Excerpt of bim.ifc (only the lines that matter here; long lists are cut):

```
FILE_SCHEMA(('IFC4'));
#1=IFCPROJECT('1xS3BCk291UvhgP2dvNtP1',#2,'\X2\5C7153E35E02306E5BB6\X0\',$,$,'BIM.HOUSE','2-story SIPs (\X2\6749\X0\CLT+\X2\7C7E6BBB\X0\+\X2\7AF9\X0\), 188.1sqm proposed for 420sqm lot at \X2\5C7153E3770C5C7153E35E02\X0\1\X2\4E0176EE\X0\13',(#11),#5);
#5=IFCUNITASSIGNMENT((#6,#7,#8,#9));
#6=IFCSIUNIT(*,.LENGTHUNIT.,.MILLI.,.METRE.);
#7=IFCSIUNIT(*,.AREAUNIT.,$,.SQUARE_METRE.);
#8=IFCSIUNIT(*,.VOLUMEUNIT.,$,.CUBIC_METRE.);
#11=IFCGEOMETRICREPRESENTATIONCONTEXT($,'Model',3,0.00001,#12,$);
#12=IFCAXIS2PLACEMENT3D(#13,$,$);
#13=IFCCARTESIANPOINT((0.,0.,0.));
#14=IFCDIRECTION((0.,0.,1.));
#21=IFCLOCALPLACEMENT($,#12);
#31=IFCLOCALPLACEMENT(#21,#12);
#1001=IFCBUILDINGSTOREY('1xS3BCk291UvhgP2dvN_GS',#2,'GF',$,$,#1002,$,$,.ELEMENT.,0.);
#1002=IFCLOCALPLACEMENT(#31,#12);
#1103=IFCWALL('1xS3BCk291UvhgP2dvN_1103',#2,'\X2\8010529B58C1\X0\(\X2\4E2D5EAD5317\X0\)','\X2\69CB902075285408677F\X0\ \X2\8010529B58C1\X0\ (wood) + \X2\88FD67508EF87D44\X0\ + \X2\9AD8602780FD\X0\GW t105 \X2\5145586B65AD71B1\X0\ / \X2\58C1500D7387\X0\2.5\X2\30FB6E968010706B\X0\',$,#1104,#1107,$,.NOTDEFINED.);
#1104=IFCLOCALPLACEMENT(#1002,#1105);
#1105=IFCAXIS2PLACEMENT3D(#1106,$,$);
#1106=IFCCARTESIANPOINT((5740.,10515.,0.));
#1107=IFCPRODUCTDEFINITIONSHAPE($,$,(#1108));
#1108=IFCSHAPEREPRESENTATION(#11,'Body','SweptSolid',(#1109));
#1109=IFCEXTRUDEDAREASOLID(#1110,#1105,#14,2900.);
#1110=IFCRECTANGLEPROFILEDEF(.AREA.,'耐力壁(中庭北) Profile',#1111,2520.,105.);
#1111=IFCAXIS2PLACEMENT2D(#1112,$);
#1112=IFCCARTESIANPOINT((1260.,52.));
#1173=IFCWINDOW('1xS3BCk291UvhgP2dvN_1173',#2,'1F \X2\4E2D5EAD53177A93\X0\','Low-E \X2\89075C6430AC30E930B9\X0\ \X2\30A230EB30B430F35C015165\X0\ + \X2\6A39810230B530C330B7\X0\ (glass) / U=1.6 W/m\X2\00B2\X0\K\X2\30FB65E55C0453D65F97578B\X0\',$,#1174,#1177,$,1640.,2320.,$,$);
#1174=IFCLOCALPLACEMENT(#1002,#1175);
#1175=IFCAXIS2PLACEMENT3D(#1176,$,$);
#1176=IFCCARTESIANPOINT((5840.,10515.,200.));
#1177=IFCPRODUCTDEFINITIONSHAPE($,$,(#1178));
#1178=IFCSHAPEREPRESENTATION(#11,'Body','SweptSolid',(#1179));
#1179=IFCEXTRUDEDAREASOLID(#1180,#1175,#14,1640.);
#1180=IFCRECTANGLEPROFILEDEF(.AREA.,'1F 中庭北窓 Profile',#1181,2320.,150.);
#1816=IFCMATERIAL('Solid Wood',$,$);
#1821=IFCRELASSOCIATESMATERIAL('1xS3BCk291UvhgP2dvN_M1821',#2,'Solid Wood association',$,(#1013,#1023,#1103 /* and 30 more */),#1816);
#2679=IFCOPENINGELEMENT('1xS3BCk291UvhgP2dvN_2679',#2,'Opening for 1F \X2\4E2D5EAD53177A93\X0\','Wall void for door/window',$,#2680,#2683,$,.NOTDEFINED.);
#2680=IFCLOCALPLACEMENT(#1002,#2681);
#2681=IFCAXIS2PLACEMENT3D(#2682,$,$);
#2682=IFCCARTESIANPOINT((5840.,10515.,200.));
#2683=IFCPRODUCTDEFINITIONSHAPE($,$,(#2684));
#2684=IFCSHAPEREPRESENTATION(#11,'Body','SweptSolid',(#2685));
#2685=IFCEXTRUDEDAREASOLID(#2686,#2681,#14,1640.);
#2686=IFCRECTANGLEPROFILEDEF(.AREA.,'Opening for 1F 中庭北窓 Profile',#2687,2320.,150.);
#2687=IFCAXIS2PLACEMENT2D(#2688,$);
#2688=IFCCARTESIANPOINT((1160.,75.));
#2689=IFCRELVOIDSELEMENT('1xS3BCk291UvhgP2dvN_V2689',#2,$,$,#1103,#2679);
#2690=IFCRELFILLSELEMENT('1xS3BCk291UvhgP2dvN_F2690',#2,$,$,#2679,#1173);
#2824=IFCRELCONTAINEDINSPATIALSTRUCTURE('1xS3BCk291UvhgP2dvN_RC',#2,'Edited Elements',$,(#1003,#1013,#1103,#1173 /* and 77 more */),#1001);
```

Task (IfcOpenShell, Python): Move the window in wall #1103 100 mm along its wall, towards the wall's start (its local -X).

```python
import ifcopenshell
import ifcopenshell.api.geometry
import ifcopenshell.util.placement
import ifcopenshell.util.unit

model = ifcopenshell.open("bim.ifc")
unit_scale = ifcopenshell.util.unit.calculate_unit_scale(model)

window = model.by_guid("1xS3BCk291UvhgP2dvN_1173")
opening = window.FillsVoids[0].RelatingOpeningElement
wall = opening.VoidsElements[0].RelatingBuildingElement

wall_matrix = ifcopenshell.util.placement.get_local_placement(wall.ObjectPlacement)
shift = wall_matrix[:3, 0] * -0.1 / unit_scale
before = ifcopenshell.util.placement.get_local_placement(window.ObjectPlacement)[:3, 3].copy()

# The window is not placed relative to its opening, so move both.
for product in (opening, window):
    matrix = ifcopenshell.util.placement.get_local_placement(product.ObjectPlacement)
    matrix[:3, 3] += shift
    ifcopenshell.api.geometry.edit_object_placement(model, product=product, matrix=matrix, is_si=False)

after = ifcopenshell.util.placement.get_local_placement(window.ObjectPlacement)[:3, 3]
print("window moved by", (after - before).round(3) + 0.0)

model.write("bim_v2.ifc")
```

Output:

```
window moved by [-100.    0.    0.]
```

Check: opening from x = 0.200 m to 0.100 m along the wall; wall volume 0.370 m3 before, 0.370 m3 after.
